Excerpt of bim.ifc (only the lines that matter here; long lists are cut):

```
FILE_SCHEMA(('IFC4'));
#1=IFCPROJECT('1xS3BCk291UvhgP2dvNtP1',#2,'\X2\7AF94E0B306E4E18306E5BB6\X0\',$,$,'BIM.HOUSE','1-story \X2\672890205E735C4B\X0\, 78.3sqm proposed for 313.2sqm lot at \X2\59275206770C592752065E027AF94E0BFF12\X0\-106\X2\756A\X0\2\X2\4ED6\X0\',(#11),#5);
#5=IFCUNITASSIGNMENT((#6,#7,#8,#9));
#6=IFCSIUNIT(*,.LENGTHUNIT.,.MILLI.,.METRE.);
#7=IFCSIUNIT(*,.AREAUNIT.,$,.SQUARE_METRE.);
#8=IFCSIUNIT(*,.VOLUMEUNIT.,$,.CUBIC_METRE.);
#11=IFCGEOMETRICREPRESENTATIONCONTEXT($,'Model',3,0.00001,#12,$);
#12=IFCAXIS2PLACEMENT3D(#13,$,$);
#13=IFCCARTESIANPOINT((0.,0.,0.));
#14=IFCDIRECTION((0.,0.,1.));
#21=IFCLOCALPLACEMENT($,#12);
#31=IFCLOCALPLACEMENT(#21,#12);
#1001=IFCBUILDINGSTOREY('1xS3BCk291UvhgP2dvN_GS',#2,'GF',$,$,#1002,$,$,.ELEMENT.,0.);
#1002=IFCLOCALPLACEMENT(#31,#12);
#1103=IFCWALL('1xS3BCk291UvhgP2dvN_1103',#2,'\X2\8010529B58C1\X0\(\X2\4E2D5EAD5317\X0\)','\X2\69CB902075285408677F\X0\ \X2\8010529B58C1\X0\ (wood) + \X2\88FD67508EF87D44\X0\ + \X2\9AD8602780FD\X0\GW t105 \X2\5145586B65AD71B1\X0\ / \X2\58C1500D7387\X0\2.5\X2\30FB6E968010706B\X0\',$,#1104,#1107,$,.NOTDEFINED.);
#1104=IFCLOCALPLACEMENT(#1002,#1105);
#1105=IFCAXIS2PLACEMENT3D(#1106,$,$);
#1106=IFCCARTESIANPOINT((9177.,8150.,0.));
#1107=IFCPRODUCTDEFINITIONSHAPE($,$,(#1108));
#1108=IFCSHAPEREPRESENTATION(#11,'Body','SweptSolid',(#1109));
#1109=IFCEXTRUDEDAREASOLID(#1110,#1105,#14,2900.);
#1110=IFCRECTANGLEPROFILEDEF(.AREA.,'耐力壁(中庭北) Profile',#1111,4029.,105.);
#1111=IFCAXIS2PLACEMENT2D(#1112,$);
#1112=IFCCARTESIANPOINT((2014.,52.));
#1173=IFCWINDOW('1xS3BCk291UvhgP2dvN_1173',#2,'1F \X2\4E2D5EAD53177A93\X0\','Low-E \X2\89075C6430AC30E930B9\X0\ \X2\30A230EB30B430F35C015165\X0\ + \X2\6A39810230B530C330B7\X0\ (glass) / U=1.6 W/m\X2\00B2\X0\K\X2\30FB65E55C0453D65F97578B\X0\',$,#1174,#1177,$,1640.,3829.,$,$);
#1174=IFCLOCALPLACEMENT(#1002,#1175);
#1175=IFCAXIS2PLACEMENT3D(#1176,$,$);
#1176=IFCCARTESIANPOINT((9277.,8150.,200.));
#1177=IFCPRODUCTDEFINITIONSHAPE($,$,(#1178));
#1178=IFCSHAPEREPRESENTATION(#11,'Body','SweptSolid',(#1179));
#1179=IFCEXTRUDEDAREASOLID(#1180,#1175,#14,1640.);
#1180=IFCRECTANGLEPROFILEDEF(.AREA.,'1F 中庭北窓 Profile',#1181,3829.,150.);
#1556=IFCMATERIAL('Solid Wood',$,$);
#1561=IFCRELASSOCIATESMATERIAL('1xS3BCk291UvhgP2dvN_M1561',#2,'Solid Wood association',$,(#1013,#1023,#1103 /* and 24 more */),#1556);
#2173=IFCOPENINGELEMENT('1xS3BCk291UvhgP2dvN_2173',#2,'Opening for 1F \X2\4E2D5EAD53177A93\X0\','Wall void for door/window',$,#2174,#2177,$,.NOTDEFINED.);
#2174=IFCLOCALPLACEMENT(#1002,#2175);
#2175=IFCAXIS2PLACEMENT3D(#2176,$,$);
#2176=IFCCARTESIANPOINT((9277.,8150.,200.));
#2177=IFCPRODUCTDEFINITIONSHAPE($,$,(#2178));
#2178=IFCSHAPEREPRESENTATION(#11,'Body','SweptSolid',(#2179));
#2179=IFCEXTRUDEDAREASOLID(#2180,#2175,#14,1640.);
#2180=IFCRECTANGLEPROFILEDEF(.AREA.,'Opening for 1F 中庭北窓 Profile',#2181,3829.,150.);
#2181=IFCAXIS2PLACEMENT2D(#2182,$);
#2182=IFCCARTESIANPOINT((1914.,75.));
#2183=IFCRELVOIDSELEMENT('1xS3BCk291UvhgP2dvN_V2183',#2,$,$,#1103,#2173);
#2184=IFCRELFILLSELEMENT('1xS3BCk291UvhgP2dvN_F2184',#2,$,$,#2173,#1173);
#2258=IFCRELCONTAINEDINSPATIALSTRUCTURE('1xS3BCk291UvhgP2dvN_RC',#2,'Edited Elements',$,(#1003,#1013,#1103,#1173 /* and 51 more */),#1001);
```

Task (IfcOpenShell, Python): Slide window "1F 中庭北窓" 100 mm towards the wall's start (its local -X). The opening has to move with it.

```python
import ifcopenshell
import ifcopenshell.api.geometry
import ifcopenshell.util.placement
import ifcopenshell.util.unit

model = ifcopenshell.open("bim.ifc")
unit_scale = ifcopenshell.util.unit.calculate_unit_scale(model)

window = model.by_guid("1xS3BCk291UvhgP2dvN_1173")
opening = window.FillsVoids[0].RelatingOpeningElement
wall = opening.VoidsElements[0].RelatingBuildingElement

wall_matrix = ifcopenshell.util.placement.get_local_placement(wall.ObjectPlacement)
shift = wall_matrix[:3, 0] * -0.1 / unit_scale
before = ifcopenshell.util.placement.get_local_placement(window.ObjectPlacement)[:3, 3].copy()

# The window is not placed relative to its opening, so move both.
for product in (opening, window):
    matrix = ifcopenshell.util.placement.get_local_placement(product.ObjectPlacement)
    matrix[:3, 3] += shift
    ifcopenshell.api.geometry.edit_object_placement(model, product=product, matrix=matrix, is_si=False)

after = ifcopenshell.util.placement.get_local_placement(window.ObjectPlacement)[:3, 3]
print("window moved by", (after - before).round(3) + 0.0)

model.write("bim-out.ifc")
```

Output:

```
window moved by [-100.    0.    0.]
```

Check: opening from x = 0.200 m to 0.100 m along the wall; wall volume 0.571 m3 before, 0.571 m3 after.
